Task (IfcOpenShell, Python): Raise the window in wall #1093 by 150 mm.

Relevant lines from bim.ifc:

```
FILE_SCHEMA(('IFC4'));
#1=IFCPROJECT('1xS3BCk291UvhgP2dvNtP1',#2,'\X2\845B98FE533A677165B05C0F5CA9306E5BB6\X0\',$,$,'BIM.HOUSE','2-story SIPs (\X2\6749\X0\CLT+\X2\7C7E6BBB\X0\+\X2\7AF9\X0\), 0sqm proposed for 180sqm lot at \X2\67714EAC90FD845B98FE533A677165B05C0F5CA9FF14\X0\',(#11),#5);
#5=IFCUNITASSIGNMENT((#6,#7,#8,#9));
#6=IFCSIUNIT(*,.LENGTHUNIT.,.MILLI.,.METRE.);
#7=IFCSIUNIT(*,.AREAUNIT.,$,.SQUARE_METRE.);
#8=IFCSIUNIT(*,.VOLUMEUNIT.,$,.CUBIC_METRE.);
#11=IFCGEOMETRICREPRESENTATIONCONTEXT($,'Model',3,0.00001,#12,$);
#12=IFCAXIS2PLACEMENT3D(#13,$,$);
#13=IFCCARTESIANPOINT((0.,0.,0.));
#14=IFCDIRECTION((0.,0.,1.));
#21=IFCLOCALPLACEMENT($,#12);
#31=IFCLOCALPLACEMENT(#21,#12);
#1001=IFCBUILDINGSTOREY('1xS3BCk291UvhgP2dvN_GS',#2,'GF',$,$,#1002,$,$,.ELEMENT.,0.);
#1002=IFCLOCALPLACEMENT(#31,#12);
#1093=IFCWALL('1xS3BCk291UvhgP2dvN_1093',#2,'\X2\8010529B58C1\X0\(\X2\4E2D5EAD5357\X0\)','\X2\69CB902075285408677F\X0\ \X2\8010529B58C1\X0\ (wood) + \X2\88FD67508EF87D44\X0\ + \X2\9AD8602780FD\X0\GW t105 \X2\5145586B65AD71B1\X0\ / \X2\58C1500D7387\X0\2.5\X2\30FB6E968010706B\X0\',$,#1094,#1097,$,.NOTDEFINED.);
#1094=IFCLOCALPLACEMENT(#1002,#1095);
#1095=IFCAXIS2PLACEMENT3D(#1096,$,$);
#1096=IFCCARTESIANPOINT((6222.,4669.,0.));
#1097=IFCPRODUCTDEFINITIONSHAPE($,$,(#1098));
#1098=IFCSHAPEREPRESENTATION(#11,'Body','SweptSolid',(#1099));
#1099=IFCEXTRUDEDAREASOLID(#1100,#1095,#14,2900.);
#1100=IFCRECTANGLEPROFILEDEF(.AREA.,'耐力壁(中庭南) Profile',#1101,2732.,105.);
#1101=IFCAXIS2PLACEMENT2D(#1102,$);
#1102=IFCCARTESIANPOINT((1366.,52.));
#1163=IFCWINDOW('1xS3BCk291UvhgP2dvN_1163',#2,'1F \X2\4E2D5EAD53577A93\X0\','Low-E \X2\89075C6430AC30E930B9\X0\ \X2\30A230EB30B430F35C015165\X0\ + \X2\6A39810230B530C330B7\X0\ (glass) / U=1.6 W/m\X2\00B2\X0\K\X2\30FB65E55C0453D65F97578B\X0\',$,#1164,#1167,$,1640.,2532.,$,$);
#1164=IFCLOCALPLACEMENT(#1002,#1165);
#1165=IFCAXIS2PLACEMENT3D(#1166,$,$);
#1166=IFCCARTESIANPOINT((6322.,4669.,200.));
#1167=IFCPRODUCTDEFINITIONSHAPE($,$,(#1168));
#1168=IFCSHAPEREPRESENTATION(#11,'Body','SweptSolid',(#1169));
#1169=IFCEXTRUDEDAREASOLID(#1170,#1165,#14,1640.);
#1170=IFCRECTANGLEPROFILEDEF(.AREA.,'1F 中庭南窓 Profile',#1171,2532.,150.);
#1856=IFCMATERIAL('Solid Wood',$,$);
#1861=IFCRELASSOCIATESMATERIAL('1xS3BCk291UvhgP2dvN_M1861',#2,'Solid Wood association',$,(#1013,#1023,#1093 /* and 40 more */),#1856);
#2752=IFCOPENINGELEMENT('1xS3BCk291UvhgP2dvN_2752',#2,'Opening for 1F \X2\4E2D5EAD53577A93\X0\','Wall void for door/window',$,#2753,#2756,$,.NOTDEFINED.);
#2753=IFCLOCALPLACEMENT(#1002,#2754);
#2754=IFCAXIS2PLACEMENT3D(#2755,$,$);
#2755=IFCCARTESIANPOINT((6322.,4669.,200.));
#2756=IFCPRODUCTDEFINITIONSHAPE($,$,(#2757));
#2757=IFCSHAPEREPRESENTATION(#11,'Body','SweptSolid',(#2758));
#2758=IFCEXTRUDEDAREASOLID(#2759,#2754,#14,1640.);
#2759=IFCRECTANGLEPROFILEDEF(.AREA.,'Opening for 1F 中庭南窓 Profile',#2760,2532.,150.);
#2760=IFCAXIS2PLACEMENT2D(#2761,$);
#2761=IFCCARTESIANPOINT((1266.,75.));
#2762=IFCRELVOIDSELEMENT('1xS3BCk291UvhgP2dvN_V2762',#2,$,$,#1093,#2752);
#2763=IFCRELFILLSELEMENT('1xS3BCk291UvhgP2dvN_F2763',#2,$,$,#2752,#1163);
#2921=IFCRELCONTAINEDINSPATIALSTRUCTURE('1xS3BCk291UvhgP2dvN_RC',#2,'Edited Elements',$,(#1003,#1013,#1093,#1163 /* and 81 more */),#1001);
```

```python
import numpy as np
import ifcopenshell
import ifcopenshell.api.geometry
import ifcopenshell.util.placement
import ifcopenshell.util.unit

model = ifcopenshell.open("bim.ifc")
unit_scale = ifcopenshell.util.unit.calculate_unit_scale(model)

window = model.by_id(1163)
opening = window.FillsVoids[0].RelatingOpeningElement
dz = 0.15 / unit_scale

shift = np.array([0.0, 0.0, dz])
# The window is not placed relative to its opening, so move both.
for product in (opening, window):
    matrix = ifcopenshell.util.placement.get_local_placement(product.ObjectPlacement)
    matrix[:3, 3] += shift
    ifcopenshell.api.geometry.edit_object_placement(model, product=product, matrix=matrix, is_si=False)

print(f"moved by {dz * unit_scale:+.3f} m")

model.write("bim_v2.ifc")
```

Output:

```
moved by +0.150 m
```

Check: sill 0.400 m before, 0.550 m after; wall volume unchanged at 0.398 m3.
